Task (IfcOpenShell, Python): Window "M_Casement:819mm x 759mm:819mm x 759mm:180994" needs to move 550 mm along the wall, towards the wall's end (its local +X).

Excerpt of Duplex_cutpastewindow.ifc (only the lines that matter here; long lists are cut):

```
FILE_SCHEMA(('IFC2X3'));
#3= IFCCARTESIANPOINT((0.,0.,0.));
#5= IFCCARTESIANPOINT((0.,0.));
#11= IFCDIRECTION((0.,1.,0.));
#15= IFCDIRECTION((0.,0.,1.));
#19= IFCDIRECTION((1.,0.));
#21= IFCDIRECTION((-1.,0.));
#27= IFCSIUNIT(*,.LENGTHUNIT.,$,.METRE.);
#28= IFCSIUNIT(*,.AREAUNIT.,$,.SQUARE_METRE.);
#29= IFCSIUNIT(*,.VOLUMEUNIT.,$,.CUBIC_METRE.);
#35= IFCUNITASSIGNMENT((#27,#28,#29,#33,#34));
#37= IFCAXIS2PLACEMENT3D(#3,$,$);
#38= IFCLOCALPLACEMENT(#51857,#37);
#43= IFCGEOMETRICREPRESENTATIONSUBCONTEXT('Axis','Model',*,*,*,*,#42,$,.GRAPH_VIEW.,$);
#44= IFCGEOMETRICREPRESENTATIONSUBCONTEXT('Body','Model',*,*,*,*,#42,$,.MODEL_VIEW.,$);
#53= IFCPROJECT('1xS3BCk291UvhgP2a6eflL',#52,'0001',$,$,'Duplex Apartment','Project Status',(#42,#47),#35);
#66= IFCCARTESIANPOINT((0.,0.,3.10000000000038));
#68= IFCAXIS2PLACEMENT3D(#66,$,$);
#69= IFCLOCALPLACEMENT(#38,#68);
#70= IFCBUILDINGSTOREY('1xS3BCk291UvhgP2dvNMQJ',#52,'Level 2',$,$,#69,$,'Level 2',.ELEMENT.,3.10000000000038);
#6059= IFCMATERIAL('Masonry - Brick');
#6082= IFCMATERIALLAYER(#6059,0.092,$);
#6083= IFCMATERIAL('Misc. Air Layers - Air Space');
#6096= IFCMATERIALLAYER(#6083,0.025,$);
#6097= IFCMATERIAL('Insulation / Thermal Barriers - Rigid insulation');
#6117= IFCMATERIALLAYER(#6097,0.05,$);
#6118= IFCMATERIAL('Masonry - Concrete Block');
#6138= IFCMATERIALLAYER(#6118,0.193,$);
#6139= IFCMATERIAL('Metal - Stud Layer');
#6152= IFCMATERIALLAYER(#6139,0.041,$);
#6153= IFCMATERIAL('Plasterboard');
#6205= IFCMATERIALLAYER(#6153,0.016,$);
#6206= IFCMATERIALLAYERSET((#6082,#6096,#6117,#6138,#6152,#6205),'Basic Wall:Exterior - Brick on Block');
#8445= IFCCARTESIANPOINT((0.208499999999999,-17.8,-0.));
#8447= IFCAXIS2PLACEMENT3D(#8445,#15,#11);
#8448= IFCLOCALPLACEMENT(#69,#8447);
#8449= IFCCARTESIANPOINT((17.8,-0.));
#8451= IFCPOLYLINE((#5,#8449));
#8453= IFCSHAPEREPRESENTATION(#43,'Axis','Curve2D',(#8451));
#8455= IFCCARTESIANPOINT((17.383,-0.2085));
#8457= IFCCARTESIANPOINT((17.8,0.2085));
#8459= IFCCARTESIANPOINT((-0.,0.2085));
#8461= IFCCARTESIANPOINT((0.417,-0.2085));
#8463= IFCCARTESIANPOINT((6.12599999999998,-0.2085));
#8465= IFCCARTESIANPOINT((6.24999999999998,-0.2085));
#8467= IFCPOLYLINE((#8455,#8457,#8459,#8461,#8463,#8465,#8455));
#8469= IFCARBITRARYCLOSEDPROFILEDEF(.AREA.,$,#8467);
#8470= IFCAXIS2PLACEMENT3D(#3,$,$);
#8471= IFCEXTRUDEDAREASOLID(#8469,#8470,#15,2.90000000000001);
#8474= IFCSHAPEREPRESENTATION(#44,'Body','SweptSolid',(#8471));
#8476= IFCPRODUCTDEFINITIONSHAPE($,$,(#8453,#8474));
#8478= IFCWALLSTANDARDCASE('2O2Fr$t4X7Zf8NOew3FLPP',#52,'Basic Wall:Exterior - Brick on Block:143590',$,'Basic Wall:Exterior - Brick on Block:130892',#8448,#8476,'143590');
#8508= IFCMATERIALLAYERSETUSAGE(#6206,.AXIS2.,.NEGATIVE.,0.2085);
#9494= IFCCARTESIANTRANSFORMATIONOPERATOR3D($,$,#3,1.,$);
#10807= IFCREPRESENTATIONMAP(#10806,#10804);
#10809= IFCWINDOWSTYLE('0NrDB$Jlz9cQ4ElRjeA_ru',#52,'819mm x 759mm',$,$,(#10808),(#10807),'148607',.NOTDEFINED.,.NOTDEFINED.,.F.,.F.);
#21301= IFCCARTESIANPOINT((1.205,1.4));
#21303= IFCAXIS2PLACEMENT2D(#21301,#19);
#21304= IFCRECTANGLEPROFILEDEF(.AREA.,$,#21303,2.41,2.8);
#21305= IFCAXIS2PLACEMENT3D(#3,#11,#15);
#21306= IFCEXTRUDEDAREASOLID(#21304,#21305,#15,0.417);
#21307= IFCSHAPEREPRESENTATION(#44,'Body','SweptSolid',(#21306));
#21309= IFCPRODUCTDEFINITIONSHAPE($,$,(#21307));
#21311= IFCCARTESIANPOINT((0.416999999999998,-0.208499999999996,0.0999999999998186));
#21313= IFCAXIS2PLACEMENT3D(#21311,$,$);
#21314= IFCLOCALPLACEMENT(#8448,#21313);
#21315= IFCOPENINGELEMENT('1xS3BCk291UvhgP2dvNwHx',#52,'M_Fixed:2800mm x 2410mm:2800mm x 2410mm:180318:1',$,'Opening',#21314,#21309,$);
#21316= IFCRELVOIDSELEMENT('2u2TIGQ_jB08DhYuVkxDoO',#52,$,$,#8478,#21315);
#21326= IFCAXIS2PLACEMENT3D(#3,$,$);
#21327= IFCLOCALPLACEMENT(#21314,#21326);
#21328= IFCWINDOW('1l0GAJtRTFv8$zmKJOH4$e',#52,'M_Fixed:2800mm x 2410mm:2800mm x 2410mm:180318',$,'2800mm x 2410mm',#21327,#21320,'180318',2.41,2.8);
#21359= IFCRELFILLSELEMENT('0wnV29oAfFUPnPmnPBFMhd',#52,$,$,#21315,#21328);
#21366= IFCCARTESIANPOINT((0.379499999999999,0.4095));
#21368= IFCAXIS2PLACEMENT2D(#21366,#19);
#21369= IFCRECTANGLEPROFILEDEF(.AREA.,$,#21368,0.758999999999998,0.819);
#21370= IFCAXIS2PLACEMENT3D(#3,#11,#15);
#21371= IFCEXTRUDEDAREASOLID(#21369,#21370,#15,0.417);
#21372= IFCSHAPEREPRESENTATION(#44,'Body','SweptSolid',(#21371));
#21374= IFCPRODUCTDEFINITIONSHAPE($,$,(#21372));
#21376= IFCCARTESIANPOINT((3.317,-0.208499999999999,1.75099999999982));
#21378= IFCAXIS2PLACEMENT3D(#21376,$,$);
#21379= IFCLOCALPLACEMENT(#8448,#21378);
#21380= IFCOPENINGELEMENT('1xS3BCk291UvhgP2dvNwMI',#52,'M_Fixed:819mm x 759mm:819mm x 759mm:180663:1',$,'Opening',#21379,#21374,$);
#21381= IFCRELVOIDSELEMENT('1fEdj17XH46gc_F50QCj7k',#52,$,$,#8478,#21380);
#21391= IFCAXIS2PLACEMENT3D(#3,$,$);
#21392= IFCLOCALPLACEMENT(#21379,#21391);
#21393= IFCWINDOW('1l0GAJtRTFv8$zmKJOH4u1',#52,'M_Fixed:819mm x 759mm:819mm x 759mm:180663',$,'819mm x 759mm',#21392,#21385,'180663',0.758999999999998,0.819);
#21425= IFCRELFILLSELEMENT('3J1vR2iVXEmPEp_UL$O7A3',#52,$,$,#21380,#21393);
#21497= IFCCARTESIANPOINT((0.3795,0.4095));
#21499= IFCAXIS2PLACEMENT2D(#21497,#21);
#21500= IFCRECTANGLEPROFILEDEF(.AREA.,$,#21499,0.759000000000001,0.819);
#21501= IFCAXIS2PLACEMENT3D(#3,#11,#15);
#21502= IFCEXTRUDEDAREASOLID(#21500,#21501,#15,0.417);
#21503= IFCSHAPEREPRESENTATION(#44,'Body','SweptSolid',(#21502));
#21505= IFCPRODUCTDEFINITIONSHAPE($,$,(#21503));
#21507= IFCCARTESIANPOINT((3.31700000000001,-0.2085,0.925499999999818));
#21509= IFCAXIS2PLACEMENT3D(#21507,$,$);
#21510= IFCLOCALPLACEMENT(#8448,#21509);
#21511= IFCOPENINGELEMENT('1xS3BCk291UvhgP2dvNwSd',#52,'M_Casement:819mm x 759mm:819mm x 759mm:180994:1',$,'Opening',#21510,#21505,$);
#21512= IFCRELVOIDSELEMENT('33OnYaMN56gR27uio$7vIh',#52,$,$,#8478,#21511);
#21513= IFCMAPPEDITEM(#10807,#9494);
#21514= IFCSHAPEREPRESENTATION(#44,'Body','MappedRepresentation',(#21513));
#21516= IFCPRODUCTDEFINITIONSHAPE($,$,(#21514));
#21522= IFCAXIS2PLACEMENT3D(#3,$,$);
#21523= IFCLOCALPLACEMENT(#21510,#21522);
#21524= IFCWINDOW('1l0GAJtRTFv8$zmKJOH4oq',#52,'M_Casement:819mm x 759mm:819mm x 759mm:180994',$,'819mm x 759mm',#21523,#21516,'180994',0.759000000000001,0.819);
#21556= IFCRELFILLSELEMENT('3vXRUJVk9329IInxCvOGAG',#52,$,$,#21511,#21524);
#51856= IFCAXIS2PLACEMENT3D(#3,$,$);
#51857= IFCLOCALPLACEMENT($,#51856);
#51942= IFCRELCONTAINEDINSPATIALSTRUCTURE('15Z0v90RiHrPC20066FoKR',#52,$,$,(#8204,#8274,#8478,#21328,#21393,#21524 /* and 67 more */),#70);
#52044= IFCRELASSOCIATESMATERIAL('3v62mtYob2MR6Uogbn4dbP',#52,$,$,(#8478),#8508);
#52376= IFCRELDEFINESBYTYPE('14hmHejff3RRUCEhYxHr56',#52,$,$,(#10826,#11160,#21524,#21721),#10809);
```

```python
import ifcopenshell
import ifcopenshell.api.geometry
import ifcopenshell.util.placement

model = ifcopenshell.open("Duplex_cutpastewindow.ifc")

window = model.by_guid("1l0GAJtRTFv8$zmKJOH4oq")
opening = window.FillsVoids[0].RelatingOpeningElement
wall = opening.VoidsElements[0].RelatingBuildingElement

wall_matrix = ifcopenshell.util.placement.get_local_placement(wall.ObjectPlacement)
shift = wall_matrix[:3, 0] * 0.55
before = ifcopenshell.util.placement.get_local_placement(window.ObjectPlacement)[:3, 3].copy()

# The window is placed relative to its opening, so it follows when the opening moves.
matrix = ifcopenshell.util.placement.get_local_placement(opening.ObjectPlacement)
matrix[:3, 3] += shift
ifcopenshell.api.geometry.edit_object_placement(
    model, product=opening, matrix=matrix, is_si=False, should_transform_children=True
)

after = ifcopenshell.util.placement.get_local_placement(window.ObjectPlacement)[:3, 3]
print("window moved by", (after - before).round(3) + 0.0)

model.write("Duplex_cutpastewindow_v2.ifc")
```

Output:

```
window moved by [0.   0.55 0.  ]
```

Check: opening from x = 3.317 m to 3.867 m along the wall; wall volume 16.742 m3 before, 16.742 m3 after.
